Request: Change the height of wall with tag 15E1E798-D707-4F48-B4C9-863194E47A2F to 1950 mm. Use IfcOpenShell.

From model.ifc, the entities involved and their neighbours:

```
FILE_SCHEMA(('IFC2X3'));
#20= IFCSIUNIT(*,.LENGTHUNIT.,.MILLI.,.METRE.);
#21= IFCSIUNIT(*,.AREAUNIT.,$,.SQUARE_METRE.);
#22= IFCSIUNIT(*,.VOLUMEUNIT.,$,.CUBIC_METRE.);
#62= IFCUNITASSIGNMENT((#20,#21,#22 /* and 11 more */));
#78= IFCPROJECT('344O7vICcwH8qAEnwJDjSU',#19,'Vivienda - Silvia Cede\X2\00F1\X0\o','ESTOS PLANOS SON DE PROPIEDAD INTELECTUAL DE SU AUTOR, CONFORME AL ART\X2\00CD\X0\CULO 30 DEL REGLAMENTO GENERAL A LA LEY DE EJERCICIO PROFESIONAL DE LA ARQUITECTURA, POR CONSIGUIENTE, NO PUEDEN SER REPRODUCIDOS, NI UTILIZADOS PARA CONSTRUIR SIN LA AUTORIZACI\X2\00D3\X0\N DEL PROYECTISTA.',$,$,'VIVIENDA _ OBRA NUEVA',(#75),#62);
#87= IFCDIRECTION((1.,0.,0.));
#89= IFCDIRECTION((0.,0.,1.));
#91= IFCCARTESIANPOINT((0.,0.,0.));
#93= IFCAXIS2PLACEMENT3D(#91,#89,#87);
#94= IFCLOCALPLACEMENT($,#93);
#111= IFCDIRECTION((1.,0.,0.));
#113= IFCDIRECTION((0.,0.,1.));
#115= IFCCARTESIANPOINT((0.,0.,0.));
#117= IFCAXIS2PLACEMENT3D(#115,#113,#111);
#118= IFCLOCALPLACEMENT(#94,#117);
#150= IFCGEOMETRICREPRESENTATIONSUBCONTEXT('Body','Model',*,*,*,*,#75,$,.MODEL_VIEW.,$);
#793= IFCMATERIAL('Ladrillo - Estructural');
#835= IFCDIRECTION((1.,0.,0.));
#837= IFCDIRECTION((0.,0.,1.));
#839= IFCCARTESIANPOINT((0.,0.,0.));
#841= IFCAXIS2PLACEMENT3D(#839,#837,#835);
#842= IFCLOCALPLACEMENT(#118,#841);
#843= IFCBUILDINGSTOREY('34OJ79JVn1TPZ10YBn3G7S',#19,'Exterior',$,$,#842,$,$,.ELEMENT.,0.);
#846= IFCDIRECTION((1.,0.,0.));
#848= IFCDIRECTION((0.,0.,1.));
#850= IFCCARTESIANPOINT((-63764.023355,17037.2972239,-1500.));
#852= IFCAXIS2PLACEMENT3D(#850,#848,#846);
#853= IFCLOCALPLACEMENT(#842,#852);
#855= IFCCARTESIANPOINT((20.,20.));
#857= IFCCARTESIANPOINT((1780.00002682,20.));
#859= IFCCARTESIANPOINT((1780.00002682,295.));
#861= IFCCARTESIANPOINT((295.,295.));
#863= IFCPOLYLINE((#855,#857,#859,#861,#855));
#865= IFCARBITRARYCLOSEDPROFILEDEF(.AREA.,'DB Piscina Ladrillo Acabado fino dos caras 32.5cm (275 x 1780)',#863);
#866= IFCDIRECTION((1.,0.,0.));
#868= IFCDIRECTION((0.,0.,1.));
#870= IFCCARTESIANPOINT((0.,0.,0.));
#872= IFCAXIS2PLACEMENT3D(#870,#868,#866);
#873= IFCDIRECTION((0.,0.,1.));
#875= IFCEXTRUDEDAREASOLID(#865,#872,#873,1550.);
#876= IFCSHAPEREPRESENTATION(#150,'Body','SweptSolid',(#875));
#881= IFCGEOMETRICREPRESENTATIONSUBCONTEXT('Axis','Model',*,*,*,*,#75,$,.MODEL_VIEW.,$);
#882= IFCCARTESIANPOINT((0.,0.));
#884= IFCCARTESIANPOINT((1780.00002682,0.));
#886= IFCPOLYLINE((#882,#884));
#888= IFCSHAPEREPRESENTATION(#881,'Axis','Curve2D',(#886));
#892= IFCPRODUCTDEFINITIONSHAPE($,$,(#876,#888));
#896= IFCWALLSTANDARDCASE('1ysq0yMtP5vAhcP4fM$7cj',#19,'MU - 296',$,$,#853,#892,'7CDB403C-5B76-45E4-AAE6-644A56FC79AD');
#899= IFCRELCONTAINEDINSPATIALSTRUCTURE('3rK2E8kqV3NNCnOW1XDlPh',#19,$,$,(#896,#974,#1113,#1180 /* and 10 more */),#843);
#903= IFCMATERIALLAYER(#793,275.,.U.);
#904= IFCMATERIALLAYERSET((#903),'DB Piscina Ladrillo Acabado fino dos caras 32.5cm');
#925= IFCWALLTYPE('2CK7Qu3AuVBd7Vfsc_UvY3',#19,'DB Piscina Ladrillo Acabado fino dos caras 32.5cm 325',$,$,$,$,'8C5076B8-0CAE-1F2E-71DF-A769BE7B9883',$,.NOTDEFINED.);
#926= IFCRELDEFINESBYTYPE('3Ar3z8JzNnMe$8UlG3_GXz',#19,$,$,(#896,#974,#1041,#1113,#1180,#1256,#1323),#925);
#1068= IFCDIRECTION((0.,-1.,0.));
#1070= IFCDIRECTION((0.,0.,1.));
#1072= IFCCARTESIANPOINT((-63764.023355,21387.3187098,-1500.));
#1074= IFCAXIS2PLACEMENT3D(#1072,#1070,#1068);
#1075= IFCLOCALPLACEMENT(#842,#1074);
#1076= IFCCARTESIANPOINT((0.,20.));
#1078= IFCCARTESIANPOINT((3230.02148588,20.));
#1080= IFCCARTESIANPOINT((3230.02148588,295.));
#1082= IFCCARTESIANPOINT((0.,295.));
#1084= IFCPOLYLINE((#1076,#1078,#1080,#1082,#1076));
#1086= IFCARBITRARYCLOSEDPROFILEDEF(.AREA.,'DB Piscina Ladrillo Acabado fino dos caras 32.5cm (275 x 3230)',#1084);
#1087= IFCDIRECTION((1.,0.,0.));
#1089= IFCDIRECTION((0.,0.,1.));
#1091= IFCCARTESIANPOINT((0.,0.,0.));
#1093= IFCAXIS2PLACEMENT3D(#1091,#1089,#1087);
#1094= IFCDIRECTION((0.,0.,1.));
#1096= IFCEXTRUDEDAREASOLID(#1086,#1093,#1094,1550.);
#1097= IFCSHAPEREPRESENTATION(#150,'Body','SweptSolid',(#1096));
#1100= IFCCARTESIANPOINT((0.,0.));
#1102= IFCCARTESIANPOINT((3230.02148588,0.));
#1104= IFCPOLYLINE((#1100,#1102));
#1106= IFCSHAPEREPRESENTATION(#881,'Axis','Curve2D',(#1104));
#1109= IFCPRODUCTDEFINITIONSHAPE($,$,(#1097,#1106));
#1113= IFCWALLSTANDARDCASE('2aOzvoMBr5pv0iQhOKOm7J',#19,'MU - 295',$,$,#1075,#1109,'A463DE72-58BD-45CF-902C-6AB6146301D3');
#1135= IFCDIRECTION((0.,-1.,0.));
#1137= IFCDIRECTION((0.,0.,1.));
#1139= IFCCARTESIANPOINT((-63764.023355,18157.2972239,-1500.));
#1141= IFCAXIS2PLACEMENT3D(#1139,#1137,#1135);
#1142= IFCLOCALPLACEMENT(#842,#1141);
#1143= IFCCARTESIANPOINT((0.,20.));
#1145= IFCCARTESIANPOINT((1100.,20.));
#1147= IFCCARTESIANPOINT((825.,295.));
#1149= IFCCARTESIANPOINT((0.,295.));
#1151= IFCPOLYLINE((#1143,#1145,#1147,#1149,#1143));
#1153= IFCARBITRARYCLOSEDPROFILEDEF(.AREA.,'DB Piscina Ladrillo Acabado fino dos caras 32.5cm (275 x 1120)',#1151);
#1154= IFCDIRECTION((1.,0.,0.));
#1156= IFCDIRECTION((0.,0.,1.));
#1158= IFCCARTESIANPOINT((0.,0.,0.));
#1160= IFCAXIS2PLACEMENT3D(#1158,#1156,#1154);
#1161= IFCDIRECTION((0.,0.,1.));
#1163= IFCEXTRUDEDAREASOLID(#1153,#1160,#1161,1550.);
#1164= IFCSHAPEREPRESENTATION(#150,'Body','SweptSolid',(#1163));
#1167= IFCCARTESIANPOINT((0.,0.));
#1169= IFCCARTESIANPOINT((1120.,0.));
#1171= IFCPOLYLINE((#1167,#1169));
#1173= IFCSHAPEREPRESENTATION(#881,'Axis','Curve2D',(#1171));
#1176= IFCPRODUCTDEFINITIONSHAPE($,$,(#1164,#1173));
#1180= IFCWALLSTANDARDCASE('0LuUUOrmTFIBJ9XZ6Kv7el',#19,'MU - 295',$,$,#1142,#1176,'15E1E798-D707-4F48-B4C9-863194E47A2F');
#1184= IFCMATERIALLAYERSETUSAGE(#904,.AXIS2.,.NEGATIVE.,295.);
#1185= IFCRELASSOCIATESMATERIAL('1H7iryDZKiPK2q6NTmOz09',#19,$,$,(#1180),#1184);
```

```python
import ifcopenshell
import ifcopenshell.geom
import ifcopenshell.util.representation
import ifcopenshell.util.shape

model = ifcopenshell.open("model.ifc")
settings = ifcopenshell.geom.settings()


def volume(element):
    """Net volume in cubic metres, openings subtracted."""
    shape = ifcopenshell.geom.create_shape(settings, element)
    return ifcopenshell.util.shape.get_volume(shape.geometry)


wall = model.by_guid("0LuUUOrmTFIBJ9XZ6Kv7el")
before = volume(wall)

body = ifcopenshell.util.representation.get_representation(wall, "Model", "Body")
solid = body.Items[0]
old_height = solid.Depth
solid.Depth = 1950.0
after = volume(wall)

print(f"height {old_height:g} -> {solid.Depth:g}, volume {before:.3f} -> {after:.3f} m3")

model.write("model_updated.ifc")
```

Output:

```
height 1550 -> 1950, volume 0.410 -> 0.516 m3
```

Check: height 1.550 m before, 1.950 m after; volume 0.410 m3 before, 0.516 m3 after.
